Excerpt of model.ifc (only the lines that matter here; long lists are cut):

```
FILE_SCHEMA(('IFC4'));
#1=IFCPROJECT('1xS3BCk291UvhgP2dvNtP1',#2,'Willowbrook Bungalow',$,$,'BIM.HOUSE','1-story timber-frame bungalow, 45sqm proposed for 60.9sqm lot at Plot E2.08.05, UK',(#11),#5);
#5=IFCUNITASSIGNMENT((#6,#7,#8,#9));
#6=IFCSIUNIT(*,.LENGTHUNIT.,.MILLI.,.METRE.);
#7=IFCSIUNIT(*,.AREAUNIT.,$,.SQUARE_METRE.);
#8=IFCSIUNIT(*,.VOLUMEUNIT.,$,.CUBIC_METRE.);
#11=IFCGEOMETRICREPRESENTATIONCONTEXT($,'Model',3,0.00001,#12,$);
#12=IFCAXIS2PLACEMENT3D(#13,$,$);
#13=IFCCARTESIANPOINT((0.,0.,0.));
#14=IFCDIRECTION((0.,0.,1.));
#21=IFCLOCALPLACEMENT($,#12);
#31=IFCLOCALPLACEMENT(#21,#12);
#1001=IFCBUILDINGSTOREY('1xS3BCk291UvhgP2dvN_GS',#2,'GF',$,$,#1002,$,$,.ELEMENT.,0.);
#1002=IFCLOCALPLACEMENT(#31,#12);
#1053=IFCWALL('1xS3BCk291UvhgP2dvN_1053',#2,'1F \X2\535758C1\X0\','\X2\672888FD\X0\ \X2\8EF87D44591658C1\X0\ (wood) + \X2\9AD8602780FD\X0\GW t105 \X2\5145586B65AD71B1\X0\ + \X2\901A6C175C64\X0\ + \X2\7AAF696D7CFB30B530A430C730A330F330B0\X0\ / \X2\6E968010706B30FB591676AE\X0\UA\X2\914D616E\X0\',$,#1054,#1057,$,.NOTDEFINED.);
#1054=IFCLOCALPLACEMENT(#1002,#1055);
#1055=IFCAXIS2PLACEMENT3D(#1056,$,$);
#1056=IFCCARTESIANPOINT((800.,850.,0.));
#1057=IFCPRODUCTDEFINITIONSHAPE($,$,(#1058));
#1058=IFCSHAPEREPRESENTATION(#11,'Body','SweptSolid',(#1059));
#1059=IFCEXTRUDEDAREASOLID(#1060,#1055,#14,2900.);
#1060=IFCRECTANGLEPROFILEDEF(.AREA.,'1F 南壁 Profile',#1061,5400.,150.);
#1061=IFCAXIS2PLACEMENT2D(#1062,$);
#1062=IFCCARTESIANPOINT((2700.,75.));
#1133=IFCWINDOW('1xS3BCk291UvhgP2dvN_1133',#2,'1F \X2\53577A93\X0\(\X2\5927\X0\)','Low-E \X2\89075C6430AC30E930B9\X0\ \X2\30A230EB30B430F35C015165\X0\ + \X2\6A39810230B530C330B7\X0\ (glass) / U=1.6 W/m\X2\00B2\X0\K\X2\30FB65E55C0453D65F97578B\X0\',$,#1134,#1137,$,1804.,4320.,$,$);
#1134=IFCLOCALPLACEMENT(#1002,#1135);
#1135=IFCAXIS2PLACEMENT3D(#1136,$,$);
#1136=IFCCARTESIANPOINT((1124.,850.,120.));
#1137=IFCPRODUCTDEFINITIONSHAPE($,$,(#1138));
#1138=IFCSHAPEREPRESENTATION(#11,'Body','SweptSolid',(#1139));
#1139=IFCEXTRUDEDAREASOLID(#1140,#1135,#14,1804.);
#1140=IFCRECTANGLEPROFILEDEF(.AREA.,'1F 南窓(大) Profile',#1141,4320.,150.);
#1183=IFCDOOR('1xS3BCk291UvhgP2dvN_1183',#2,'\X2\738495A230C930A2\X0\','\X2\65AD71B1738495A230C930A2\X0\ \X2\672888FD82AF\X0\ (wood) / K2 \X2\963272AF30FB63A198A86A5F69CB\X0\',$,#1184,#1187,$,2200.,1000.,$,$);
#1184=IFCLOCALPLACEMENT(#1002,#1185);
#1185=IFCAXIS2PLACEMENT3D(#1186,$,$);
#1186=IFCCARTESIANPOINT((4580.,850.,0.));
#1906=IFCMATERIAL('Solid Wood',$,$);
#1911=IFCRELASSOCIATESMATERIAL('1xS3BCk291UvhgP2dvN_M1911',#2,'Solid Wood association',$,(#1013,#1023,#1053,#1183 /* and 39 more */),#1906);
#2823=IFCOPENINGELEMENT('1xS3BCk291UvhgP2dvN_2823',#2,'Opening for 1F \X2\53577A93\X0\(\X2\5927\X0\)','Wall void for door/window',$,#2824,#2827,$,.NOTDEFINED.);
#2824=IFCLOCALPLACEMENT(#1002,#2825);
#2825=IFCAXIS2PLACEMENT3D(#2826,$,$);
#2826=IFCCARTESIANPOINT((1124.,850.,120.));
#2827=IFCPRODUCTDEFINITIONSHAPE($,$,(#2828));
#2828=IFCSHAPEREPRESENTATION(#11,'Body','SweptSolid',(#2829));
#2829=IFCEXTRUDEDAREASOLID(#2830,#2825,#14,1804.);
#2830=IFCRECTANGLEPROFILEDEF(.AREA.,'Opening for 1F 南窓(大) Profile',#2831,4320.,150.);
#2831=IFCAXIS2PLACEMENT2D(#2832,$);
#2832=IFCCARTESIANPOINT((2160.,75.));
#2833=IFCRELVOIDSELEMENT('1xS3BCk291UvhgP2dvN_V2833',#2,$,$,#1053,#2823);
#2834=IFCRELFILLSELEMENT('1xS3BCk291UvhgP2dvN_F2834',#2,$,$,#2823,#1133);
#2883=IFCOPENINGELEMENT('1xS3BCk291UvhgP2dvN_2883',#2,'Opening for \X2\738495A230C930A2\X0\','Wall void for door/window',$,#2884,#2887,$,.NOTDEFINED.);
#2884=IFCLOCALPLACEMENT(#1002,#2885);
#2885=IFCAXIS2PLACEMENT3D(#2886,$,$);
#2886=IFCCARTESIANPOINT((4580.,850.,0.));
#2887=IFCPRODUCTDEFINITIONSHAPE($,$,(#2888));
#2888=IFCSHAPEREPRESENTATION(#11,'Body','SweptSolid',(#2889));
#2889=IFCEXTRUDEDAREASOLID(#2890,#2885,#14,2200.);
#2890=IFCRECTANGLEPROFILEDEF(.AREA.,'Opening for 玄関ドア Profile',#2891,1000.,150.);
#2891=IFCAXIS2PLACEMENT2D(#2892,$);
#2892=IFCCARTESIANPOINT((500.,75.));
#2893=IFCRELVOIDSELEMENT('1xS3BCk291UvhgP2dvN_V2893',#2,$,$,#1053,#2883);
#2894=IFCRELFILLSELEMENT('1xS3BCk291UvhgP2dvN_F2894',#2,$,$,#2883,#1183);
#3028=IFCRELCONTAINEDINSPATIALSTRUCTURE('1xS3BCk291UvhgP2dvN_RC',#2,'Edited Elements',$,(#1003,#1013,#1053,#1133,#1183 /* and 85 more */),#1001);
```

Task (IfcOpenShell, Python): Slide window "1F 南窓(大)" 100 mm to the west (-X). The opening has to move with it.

```python
import ifcopenshell
import ifcopenshell.api.geometry
import ifcopenshell.util.placement
import ifcopenshell.util.unit

model = ifcopenshell.open("model.ifc")
unit_scale = ifcopenshell.util.unit.calculate_unit_scale(model)

window = model.by_guid("1xS3BCk291UvhgP2dvN_1133")
opening = window.FillsVoids[0].RelatingOpeningElement
wall = opening.VoidsElements[0].RelatingBuildingElement

wall_matrix = ifcopenshell.util.placement.get_local_placement(wall.ObjectPlacement)
shift = wall_matrix[:3, 0] * -0.1 / unit_scale
before = ifcopenshell.util.placement.get_local_placement(window.ObjectPlacement)[:3, 3].copy()

# The window is not placed relative to its opening, so move both.
for product in (opening, window):
    matrix = ifcopenshell.util.placement.get_local_placement(product.ObjectPlacement)
    matrix[:3, 3] += shift
    ifcopenshell.api.geometry.edit_object_placement(model, product=product, matrix=matrix, is_si=False)

after = ifcopenshell.util.placement.get_local_placement(window.ObjectPlacement)[:3, 3]
print("window moved by", (after - before).round(3) + 0.0)

model.write("model_edited.ifc")
```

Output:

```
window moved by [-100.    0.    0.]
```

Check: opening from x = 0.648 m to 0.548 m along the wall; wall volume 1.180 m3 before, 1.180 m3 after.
